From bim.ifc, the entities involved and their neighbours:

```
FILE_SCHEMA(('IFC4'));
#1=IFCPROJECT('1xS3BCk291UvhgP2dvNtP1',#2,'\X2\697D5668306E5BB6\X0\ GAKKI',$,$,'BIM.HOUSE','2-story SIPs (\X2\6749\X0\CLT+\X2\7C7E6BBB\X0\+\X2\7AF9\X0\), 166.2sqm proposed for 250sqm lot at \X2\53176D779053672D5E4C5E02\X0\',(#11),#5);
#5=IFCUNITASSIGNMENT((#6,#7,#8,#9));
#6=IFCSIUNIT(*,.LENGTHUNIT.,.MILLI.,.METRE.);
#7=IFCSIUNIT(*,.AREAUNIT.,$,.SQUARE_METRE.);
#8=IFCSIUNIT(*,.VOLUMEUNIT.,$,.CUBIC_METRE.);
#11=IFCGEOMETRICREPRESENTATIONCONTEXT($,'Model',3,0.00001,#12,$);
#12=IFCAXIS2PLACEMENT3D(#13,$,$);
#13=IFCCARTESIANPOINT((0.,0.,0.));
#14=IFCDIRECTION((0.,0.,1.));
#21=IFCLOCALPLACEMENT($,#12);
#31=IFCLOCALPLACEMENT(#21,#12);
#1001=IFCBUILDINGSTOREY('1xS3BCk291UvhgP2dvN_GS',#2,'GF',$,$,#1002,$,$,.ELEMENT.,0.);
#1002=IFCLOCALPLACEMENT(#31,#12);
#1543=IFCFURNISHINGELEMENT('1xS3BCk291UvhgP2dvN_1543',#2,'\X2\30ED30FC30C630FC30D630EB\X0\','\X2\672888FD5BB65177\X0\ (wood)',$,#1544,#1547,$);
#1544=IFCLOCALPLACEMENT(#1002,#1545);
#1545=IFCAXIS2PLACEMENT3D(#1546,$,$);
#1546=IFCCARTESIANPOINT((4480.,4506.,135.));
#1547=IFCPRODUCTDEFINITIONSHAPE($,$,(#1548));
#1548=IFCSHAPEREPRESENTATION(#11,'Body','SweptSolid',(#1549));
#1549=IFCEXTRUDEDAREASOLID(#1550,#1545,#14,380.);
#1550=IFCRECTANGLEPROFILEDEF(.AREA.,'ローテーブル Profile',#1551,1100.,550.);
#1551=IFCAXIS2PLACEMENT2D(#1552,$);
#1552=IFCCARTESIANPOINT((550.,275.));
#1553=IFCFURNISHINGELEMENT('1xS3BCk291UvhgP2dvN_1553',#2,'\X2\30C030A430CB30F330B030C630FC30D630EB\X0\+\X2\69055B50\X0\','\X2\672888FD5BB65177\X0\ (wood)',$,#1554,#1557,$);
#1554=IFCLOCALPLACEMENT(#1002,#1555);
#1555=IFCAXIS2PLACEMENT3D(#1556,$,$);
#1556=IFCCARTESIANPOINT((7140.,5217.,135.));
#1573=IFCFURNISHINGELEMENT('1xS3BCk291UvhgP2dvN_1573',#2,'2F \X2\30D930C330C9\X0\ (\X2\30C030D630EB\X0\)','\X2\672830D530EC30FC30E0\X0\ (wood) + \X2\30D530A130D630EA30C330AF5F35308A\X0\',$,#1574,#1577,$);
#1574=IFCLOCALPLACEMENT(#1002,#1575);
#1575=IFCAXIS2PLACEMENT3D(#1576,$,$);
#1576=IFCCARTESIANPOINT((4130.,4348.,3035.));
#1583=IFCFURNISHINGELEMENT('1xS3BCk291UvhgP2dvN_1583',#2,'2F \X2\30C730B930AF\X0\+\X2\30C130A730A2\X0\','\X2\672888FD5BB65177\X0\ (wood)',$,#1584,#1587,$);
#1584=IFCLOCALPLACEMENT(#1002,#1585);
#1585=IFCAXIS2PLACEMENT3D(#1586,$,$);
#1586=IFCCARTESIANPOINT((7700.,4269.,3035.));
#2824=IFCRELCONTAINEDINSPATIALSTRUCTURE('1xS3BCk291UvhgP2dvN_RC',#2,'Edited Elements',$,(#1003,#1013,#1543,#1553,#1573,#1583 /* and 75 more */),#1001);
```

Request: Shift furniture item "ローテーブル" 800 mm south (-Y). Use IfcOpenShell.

```python
import ifcopenshell
import ifcopenshell.api.geometry
import ifcopenshell.util.placement
import ifcopenshell.util.unit

model = ifcopenshell.open("bim.ifc")
unit_scale = ifcopenshell.util.unit.calculate_unit_scale(model)

item = model.by_guid("1xS3BCk291UvhgP2dvN_1543")
matrix = ifcopenshell.util.placement.get_local_placement(item.ObjectPlacement)
matrix[1, 3] -= 0.8 / unit_scale
ifcopenshell.api.geometry.edit_object_placement(model, product=item, matrix=matrix, is_si=False)

print(ifcopenshell.util.placement.get_local_placement(item.ObjectPlacement).round(3) + 0.0)

model.write("bim_edited.ifc")
```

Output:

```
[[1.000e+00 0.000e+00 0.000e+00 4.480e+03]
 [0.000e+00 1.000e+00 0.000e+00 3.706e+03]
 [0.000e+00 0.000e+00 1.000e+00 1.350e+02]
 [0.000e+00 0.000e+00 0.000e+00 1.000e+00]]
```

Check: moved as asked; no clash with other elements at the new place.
